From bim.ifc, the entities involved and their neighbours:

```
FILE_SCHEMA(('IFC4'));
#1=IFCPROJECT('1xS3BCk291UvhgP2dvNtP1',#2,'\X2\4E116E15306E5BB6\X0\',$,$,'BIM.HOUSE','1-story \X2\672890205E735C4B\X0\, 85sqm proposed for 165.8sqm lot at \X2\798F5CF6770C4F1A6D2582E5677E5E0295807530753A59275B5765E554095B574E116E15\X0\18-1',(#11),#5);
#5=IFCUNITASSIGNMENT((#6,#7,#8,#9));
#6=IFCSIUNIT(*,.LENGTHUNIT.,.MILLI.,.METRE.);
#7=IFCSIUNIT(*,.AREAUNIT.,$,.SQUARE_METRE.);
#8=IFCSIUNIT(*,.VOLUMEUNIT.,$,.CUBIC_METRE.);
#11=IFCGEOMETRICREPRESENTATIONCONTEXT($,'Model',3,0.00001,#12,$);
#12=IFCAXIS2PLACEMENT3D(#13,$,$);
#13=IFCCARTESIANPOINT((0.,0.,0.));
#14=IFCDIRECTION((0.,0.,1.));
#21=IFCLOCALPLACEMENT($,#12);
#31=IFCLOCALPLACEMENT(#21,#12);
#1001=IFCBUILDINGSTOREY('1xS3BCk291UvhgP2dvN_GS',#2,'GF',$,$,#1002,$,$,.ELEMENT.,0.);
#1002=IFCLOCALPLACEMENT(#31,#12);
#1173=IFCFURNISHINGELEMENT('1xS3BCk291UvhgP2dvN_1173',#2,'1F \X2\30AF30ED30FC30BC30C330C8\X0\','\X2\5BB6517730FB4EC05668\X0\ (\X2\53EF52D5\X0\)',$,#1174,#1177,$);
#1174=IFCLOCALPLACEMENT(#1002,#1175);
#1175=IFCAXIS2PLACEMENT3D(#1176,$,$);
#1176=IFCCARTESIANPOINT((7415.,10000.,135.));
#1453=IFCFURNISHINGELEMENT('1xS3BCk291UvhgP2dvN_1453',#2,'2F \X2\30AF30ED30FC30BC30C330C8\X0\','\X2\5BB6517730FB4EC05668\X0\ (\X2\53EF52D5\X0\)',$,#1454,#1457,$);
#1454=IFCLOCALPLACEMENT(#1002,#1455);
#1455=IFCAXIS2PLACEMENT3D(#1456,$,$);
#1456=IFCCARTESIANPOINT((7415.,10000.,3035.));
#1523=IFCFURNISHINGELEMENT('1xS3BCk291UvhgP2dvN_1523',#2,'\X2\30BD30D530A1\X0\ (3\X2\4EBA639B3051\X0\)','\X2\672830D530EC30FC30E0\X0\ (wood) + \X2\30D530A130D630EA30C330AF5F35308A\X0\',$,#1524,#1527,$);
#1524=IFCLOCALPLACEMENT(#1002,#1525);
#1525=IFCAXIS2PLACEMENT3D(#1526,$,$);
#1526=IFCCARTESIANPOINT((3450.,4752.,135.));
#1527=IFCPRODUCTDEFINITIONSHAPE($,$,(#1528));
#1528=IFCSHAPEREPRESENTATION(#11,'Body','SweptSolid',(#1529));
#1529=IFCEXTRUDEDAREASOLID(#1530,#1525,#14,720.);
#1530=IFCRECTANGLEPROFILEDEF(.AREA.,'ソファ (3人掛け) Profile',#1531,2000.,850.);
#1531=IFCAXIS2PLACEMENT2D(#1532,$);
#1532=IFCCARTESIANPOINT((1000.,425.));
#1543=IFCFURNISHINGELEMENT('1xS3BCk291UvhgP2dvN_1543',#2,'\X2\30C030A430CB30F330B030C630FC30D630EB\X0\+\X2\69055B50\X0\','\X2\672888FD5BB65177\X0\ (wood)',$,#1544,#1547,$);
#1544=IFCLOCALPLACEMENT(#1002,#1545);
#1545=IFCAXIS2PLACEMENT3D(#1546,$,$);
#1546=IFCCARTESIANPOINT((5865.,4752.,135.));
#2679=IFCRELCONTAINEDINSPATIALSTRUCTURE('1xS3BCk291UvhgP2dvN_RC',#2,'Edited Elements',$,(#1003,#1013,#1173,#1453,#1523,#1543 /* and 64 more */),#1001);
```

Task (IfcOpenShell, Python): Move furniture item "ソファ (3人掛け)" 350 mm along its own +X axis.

```python
import ifcopenshell
import ifcopenshell.api.geometry
import ifcopenshell.util.placement
import ifcopenshell.util.unit

model = ifcopenshell.open("bim.ifc")
unit_scale = ifcopenshell.util.unit.calculate_unit_scale(model)

item = model.by_guid("1xS3BCk291UvhgP2dvN_1523")
matrix = ifcopenshell.util.placement.get_local_placement(item.ObjectPlacement)
matrix[:3, 3] += matrix[:3, 0] * 0.35 / unit_scale
ifcopenshell.api.geometry.edit_object_placement(model, product=item, matrix=matrix, is_si=False)

print(ifcopenshell.util.placement.get_local_placement(item.ObjectPlacement).round(3) + 0.0)

model.write("bim-out.ifc")
```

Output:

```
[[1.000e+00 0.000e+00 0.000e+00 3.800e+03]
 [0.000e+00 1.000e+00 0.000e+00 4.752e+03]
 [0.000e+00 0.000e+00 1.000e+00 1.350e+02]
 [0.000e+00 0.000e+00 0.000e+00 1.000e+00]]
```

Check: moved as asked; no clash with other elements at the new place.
